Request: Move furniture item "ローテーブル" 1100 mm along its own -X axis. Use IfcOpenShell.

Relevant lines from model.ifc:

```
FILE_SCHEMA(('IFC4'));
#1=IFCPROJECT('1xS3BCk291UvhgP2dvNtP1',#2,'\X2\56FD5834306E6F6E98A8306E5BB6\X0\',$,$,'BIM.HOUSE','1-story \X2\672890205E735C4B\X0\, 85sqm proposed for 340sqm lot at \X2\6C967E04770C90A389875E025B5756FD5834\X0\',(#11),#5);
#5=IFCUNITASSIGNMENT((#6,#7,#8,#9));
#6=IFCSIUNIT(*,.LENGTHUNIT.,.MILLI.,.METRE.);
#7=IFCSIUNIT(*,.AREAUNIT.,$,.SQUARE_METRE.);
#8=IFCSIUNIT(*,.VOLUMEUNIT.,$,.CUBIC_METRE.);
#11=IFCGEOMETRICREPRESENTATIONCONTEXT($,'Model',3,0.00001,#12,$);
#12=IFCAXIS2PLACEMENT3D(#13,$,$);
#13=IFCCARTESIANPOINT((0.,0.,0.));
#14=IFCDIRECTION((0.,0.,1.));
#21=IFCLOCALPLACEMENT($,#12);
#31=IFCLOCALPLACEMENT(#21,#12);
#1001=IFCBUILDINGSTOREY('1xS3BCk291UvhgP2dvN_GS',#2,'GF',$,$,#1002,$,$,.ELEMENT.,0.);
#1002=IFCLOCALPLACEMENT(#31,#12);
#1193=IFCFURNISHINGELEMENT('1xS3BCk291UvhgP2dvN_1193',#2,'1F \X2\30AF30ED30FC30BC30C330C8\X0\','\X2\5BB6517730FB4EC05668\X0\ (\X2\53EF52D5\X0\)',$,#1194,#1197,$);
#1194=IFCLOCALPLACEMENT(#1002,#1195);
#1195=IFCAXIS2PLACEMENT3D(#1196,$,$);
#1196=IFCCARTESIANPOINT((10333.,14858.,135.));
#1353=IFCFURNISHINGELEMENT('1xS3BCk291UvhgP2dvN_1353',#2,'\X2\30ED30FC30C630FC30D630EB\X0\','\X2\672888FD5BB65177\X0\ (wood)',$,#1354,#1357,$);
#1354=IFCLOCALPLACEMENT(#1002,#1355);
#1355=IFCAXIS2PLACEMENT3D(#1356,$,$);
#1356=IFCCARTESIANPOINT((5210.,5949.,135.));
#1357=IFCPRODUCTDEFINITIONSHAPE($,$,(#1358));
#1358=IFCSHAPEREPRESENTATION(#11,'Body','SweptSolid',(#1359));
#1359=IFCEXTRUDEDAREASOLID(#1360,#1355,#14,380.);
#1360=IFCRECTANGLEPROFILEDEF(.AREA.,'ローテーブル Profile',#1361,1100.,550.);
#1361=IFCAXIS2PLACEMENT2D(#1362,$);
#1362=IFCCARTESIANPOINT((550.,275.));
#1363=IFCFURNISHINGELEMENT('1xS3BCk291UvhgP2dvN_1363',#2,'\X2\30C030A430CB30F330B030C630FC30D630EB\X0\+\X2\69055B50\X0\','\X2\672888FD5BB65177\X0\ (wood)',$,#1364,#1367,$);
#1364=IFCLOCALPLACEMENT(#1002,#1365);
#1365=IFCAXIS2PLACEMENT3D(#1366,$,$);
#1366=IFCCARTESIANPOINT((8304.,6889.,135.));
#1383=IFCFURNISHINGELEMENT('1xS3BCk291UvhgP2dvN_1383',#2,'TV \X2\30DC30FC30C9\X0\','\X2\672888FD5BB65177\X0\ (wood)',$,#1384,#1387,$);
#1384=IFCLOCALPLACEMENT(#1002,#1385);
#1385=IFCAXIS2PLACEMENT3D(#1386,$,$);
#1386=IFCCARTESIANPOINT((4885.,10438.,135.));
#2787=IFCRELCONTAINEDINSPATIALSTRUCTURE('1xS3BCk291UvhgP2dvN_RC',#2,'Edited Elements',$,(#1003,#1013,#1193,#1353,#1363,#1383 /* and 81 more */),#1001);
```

```python
import ifcopenshell
import ifcopenshell.api.geometry
import ifcopenshell.util.placement
import ifcopenshell.util.unit

model = ifcopenshell.open("model.ifc")
unit_scale = ifcopenshell.util.unit.calculate_unit_scale(model)

item = model.by_guid("1xS3BCk291UvhgP2dvN_1353")
matrix = ifcopenshell.util.placement.get_local_placement(item.ObjectPlacement)
matrix[:3, 3] -= matrix[:3, 0] * 1.1 / unit_scale
ifcopenshell.api.geometry.edit_object_placement(model, product=item, matrix=matrix, is_si=False)

print(ifcopenshell.util.placement.get_local_placement(item.ObjectPlacement).round(3) + 0.0)

model.write("model_updated.ifc")
```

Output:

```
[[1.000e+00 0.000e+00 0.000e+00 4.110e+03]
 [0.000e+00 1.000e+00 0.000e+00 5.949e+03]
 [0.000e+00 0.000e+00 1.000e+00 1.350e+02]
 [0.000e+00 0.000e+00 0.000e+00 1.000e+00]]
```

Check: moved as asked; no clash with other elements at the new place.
